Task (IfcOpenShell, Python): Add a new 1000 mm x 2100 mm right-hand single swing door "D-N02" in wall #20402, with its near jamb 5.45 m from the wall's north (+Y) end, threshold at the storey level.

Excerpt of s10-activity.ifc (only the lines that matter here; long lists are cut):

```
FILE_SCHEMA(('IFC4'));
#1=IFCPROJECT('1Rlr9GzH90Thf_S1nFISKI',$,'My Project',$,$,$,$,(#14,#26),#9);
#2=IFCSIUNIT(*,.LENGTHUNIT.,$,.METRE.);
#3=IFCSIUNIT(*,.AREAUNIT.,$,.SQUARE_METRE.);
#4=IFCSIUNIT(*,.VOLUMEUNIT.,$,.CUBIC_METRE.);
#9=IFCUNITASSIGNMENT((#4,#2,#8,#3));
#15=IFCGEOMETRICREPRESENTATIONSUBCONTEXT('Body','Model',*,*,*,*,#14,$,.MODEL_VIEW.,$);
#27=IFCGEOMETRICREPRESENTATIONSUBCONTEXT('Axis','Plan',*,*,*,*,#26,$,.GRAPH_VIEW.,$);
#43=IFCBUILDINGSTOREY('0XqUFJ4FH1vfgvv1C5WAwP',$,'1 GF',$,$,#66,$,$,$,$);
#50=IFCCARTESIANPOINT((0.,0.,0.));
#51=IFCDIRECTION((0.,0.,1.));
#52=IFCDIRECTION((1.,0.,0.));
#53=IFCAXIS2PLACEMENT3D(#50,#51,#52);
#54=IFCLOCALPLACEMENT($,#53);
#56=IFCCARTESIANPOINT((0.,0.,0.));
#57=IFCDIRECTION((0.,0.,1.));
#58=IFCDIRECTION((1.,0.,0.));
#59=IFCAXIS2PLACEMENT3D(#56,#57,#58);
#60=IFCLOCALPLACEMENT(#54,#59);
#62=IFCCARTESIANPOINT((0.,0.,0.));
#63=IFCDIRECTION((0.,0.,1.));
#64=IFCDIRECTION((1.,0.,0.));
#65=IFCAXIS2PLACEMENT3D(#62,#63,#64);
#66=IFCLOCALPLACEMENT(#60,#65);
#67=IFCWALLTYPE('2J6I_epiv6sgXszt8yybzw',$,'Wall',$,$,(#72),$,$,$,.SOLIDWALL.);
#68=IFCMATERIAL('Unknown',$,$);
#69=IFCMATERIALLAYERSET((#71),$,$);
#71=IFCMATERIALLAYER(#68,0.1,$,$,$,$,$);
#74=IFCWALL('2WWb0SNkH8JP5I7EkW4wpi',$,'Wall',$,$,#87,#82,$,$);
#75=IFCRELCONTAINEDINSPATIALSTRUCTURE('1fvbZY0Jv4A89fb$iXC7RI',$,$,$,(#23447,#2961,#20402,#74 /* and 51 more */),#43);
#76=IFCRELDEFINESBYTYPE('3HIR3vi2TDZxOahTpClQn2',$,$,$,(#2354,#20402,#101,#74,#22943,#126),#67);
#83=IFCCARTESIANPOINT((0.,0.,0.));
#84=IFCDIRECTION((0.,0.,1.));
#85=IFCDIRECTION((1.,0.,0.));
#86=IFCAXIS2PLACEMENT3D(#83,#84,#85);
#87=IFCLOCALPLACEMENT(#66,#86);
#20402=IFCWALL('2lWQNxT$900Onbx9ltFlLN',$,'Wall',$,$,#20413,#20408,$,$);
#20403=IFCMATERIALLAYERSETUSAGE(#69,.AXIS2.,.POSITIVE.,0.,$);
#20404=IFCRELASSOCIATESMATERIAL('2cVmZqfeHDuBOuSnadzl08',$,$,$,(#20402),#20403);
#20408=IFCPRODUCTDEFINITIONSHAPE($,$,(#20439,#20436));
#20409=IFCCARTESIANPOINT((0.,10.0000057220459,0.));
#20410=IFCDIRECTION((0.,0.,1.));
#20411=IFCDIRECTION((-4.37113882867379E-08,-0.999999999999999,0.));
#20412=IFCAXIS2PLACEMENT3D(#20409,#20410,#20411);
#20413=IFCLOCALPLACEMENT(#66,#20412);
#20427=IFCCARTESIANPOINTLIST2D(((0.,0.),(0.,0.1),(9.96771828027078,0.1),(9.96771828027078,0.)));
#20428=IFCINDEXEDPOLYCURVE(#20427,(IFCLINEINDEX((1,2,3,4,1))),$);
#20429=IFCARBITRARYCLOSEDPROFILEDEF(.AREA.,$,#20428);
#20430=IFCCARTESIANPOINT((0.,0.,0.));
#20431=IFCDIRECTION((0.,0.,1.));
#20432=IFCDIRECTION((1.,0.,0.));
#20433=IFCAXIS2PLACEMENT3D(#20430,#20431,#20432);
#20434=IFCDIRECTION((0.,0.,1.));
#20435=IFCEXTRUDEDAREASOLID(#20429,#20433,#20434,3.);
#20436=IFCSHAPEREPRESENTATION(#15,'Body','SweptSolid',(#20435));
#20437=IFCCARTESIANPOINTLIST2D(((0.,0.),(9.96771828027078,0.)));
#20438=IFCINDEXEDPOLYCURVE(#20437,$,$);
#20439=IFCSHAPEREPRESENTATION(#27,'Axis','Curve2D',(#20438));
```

```python
import numpy as np
import ifcopenshell
import ifcopenshell.api.feature
import ifcopenshell.api.geometry
import ifcopenshell.api.root
import ifcopenshell.api.spatial
import ifcopenshell.geom
import ifcopenshell.util.element
import ifcopenshell.util.placement
import ifcopenshell.util.representation
import ifcopenshell.util.shape
import ifcopenshell.util.unit

model = ifcopenshell.open("s10-activity.ifc")
unit_scale = ifcopenshell.util.unit.calculate_unit_scale(model)
settings = ifcopenshell.geom.settings()


def volume(element):
    """Net volume in cubic metres, openings subtracted."""
    shape = ifcopenshell.geom.create_shape(settings, element)
    return ifcopenshell.util.shape.get_volume(shape.geometry)


wall = model.by_guid("2lWQNxT$900Onbx9ltFlLN")
storey = ifcopenshell.util.element.get_container(wall, ifc_class="IfcBuildingStorey")
context = ifcopenshell.util.representation.get_context(model, "Model", "Body", "MODEL_VIEW")
before = volume(wall)

width, height, from_end, sill = 1, 2.1, 5.45, 0.0  # metres

# The wall runs along its own X axis, and the end named is its -X end.
wall_shape = ifcopenshell.geom.create_shape(settings, wall)
x, y, z = ifcopenshell.util.shape.get_vertices(wall_shape.geometry).T
start = x.min() + from_end
face, thickness = float(y.min()), float(y.max() - y.min())
wall_matrix = ifcopenshell.util.placement.get_local_placement(wall.ObjectPlacement)
level = ifcopenshell.util.placement.get_local_placement(storey.ObjectPlacement)[2, 3]


def in_wall(x, y):
    """Placement at x, y metres in the wall's axes, at sill height."""
    matrix = wall_matrix.copy()
    matrix[:, 3] = wall_matrix @ np.array([x / unit_scale, y / unit_scale, 0.0, 1.0])
    matrix[2, 3] = level + sill / unit_scale
    return matrix


# Opening: a box that overshoots both wall faces by 50 mm.
opening = ifcopenshell.api.root.create_entity(model, ifc_class="IfcOpeningElement", predefined_type="OPENING")
box = ifcopenshell.api.geometry.add_wall_representation(
    model, context=context, length=width, height=height, thickness=thickness + 0.1
)
ifcopenshell.api.geometry.assign_representation(model, product=opening, representation=box)
ifcopenshell.api.geometry.edit_object_placement(model, product=opening, matrix=in_wall(start, face - 0.05), is_si=False)
ifcopenshell.api.feature.add_feature(model, feature=opening, element=wall)

door = ifcopenshell.api.root.create_entity(model, ifc_class="IfcDoor", name="D-N02", predefined_type="DOOR")
door.OverallWidth, door.OverallHeight = width / unit_scale, height / unit_scale
door.OperationType = "SINGLE_SWING_RIGHT"
body = ifcopenshell.api.geometry.add_door_representation(
    model,
    context=context,
    overall_width=door.OverallWidth,
    overall_height=door.OverallHeight,
    operation_type="SINGLE_SWING_RIGHT",
    lining_properties={"LiningDepth": thickness / unit_scale, "ThresholdDepth": thickness / unit_scale},
)
ifcopenshell.api.geometry.assign_representation(model, product=door, representation=body)
ifcopenshell.api.spatial.assign_container(model, products=[door], relating_structure=storey)
ifcopenshell.api.feature.add_filling(model, opening=opening, element=door)

# The lining spans the wall, so the door starts at the wall face.
ifcopenshell.api.geometry.edit_object_placement(model, product=door, matrix=in_wall(start, face), is_si=False)

after = volume(wall)

print(f"wall volume {before:.3f} -> {after:.3f} m3")

model.write("s10-activity_edited.ifc")
```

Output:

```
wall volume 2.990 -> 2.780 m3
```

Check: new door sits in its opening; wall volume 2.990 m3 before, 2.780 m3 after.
